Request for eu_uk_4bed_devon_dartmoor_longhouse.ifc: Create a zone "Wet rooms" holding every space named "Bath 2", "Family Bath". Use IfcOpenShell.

First a look at what the model holds.

```python
import ifcopenshell

model = ifcopenshell.open("eu_uk_4bed_devon_dartmoor_longhouse.ifc")
print(model.schema)
seen = {}
for space in model.by_type("IfcSpace"):
    seen[space.LongName] = seen.get(space.LongName, 0) + 1
for name, count in sorted(seen.items(), key=str):
    print(count, "x", name)
print("zones:", [z.Name for z in model.by_type("IfcZone")][:20])
```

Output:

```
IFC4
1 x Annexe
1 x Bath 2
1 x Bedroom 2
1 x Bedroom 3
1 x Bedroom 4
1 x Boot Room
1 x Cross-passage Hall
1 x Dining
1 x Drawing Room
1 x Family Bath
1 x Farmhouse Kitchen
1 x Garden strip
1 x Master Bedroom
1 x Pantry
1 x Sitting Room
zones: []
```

```python
import ifcopenshell
import ifcopenshell.api.group
import ifcopenshell.api.root

model = ifcopenshell.open("eu_uk_4bed_devon_dartmoor_longhouse.ifc")

names = {"Bath 2", "Family Bath"}
spaces = [s for s in model.by_type("IfcSpace") if s.LongName in names]

zone = ifcopenshell.api.root.create_entity(model, ifc_class="IfcZone", name="Wet rooms")
ifcopenshell.api.group.assign_group(model, products=spaces, group=zone)
print(len(spaces), "spaces in", zone.Name)

model.write("eu_uk_4bed_devon_dartmoor_longhouse_v2.ifc")
```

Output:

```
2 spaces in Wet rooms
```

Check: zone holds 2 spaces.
